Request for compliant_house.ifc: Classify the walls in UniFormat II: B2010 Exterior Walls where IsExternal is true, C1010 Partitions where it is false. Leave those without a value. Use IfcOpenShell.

First a look at what the model holds.

```python
import ifcopenshell
import ifcopenshell.util.element

model = ifcopenshell.open("compliant_house.ifc")
print(model.schema)
print("classifications:", [c.Name for c in model.by_type("IfcClassification")])
values = [ifcopenshell.util.element.get_pset(e, "Pset_WallCommon", "IsExternal") for e in model.by_type("IfcWall")]
for value in (True, False, None):
    print("IsExternal", value, values.count(value))
```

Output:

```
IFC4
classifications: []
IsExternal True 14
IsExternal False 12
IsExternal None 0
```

```python
import ifcopenshell
import ifcopenshell.api.classification
import ifcopenshell.util.element

model = ifcopenshell.open("compliant_house.ifc")

system = ifcopenshell.api.classification.add_classification(model, classification="UniFormat II")

walls = model.by_type("IfcWall")
external = {e: ifcopenshell.util.element.get_pset(e, "Pset_WallCommon", "IsExternal") for e in walls}
for flag, code, name in ((True, "B2010", "Exterior Walls"), (False, "C1010", "Partitions")):
    products = [e for e in walls if external[e] is flag]
    ifcopenshell.api.classification.add_reference(
        model, products=products, classification=system, identification=code, name=name
    )
    print(code, len(products))

model.write("compliant_house_rev.ifc")
```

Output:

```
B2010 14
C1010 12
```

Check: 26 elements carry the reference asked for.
